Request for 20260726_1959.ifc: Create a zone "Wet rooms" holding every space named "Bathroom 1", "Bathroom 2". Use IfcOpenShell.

First a look at what the model holds.

```python
import ifcopenshell

model = ifcopenshell.open("20260726_1959.ifc")
print(model.schema)
seen = {}
for space in model.by_type("IfcSpace"):
    seen[space.LongName] = seen.get(space.LongName, 0) + 1
for name, count in sorted(seen.items(), key=str):
    print(count, "x", name)
print("zones:", [z.Name for z in model.by_type("IfcZone")][:20])
```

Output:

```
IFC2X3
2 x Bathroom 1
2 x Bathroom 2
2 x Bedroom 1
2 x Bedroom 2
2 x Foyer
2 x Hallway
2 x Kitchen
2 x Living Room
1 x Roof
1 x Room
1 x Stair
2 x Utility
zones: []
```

```python
import ifcopenshell
import ifcopenshell.api.group
import ifcopenshell.api.root

model = ifcopenshell.open("20260726_1959.ifc")

names = {"Bathroom 1", "Bathroom 2"}
spaces = [s for s in model.by_type("IfcSpace") if s.LongName in names]

zone = ifcopenshell.api.root.create_entity(model, ifc_class="IfcZone", name="Wet rooms")
ifcopenshell.api.group.assign_group(model, products=spaces, group=zone)
print(len(spaces), "spaces in", zone.Name)

model.write("20260726_1959_updated.ifc")
```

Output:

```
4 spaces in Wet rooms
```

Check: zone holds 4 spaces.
